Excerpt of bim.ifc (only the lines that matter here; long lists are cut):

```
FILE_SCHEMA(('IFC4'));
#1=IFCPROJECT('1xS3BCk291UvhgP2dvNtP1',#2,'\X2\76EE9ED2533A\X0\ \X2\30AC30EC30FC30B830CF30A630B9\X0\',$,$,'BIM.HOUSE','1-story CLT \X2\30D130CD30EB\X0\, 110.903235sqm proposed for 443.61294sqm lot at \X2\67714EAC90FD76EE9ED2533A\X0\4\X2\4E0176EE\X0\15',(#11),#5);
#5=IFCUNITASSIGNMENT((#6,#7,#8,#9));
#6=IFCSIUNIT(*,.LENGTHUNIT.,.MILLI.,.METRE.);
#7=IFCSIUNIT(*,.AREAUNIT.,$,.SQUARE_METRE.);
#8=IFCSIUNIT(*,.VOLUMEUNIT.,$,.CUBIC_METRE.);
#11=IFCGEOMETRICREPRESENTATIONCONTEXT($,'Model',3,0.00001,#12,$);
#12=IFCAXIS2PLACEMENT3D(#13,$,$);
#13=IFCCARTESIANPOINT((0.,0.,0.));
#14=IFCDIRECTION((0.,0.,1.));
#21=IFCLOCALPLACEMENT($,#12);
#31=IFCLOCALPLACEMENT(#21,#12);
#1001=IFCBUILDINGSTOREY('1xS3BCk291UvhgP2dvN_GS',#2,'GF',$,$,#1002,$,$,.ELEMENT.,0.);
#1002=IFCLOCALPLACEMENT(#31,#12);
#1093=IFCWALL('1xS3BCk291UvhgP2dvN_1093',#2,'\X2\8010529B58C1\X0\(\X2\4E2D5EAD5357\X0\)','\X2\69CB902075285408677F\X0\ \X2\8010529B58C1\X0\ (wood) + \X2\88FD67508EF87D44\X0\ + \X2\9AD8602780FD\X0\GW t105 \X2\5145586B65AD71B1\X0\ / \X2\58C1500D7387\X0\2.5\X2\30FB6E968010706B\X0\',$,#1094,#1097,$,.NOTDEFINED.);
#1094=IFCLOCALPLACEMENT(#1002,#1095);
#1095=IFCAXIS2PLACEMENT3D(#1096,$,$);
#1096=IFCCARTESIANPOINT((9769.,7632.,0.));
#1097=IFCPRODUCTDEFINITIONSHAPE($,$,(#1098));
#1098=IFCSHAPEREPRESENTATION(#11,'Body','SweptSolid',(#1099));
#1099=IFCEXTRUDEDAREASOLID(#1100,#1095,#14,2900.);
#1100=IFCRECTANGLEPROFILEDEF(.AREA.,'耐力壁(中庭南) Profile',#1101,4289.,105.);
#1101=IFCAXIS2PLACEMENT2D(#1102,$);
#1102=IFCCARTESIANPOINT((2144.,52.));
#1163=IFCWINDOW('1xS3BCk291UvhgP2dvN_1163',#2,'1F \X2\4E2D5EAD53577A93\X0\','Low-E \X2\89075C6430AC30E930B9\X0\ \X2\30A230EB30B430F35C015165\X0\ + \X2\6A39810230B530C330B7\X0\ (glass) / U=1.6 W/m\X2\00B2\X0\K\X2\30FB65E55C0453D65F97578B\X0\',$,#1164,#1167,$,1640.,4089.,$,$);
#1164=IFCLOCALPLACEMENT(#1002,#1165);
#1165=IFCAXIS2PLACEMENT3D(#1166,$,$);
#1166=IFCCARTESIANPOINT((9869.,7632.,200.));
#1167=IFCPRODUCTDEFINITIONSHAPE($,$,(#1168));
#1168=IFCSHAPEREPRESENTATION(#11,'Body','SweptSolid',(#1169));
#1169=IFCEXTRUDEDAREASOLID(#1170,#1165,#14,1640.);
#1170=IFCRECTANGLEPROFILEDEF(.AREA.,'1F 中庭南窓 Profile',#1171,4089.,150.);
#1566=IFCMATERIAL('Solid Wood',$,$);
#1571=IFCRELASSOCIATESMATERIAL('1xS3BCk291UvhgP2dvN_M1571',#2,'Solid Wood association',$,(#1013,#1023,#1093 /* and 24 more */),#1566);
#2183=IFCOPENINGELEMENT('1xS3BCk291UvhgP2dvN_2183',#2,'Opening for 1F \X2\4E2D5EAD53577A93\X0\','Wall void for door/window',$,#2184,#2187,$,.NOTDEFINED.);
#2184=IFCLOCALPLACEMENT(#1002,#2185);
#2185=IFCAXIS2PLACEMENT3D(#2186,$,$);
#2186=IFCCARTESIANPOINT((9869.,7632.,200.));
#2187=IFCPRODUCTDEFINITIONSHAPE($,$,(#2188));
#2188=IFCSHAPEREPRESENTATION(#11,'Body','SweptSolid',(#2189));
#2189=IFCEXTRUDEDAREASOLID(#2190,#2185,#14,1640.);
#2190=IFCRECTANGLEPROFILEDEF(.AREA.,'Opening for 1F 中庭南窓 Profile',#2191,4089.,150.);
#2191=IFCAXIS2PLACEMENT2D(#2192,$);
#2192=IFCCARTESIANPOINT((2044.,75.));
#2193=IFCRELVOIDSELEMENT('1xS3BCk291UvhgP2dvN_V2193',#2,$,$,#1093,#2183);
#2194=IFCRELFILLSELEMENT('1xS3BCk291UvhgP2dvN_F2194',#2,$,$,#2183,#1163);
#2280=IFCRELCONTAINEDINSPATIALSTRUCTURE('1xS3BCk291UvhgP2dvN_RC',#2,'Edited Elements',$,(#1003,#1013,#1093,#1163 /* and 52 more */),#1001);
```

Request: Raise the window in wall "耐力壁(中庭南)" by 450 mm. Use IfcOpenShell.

```python
import numpy as np
import ifcopenshell
import ifcopenshell.api.geometry
import ifcopenshell.util.placement
import ifcopenshell.util.unit

model = ifcopenshell.open("bim.ifc")
unit_scale = ifcopenshell.util.unit.calculate_unit_scale(model)

window = model.by_guid("1xS3BCk291UvhgP2dvN_1163")
opening = window.FillsVoids[0].RelatingOpeningElement
dz = 450.0

shift = np.array([0.0, 0.0, dz])
# The window is not placed relative to its opening, so move both.
for product in (opening, window):
    matrix = ifcopenshell.util.placement.get_local_placement(product.ObjectPlacement)
    matrix[:3, 3] += shift
    ifcopenshell.api.geometry.edit_object_placement(model, product=product, matrix=matrix, is_si=False)

print(f"moved by {dz * unit_scale:+.3f} m")

model.write("bim-out.ifc")
```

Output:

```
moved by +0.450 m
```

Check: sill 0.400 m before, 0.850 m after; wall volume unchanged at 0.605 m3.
